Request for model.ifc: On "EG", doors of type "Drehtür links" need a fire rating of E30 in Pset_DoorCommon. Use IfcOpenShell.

First a look at what the model holds.

```python
import ifcopenshell
import ifcopenshell.util.element

model = ifcopenshell.open("model.ifc")
print(model.schema)
storey = next(s for s in model.by_type("IfcBuildingStorey") if s.Name == "EG")
doors = [e for e in ifcopenshell.util.element.get_decomposition(storey) if e.is_a("IfcDoor")]
seen = {}
for e in doors:
    element_type = ifcopenshell.util.element.get_type(e)
    key = (element_type.Name if element_type != e and element_type else None, ifcopenshell.util.element.get_pset(e, "Pset_DoorCommon", "FireRating"))
    seen[key] = seen.get(key, 0) + 1
for (name, value), count in sorted(seen.items(), key=str):
    print(count, "x", name, "|", value)
```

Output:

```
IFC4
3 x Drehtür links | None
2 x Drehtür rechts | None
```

```python
import ifcopenshell
import ifcopenshell.api.pset
import ifcopenshell.util.element

model = ifcopenshell.open("model.ifc")

storey = next(s for s in model.by_type("IfcBuildingStorey") if s.Name == "EG")
doors = [e for e in ifcopenshell.util.element.get_decomposition(storey) if e.is_a("IfcDoor")]

count = 0
for e in doors:
    element_type = ifcopenshell.util.element.get_type(e)
    if element_type in (None, e) or element_type.Name != "Drehtür links":
        continue
    # add_pset returns the element's existing set when there is one.
    pset = ifcopenshell.api.pset.add_pset(model, product=e, name="Pset_DoorCommon")
    ifcopenshell.api.pset.edit_pset(model, pset=pset, properties={"FireRating": "E30"})
    count += 1

print(count, "doors updated")

model.write("model_edited.ifc")
```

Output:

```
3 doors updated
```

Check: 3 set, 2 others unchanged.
